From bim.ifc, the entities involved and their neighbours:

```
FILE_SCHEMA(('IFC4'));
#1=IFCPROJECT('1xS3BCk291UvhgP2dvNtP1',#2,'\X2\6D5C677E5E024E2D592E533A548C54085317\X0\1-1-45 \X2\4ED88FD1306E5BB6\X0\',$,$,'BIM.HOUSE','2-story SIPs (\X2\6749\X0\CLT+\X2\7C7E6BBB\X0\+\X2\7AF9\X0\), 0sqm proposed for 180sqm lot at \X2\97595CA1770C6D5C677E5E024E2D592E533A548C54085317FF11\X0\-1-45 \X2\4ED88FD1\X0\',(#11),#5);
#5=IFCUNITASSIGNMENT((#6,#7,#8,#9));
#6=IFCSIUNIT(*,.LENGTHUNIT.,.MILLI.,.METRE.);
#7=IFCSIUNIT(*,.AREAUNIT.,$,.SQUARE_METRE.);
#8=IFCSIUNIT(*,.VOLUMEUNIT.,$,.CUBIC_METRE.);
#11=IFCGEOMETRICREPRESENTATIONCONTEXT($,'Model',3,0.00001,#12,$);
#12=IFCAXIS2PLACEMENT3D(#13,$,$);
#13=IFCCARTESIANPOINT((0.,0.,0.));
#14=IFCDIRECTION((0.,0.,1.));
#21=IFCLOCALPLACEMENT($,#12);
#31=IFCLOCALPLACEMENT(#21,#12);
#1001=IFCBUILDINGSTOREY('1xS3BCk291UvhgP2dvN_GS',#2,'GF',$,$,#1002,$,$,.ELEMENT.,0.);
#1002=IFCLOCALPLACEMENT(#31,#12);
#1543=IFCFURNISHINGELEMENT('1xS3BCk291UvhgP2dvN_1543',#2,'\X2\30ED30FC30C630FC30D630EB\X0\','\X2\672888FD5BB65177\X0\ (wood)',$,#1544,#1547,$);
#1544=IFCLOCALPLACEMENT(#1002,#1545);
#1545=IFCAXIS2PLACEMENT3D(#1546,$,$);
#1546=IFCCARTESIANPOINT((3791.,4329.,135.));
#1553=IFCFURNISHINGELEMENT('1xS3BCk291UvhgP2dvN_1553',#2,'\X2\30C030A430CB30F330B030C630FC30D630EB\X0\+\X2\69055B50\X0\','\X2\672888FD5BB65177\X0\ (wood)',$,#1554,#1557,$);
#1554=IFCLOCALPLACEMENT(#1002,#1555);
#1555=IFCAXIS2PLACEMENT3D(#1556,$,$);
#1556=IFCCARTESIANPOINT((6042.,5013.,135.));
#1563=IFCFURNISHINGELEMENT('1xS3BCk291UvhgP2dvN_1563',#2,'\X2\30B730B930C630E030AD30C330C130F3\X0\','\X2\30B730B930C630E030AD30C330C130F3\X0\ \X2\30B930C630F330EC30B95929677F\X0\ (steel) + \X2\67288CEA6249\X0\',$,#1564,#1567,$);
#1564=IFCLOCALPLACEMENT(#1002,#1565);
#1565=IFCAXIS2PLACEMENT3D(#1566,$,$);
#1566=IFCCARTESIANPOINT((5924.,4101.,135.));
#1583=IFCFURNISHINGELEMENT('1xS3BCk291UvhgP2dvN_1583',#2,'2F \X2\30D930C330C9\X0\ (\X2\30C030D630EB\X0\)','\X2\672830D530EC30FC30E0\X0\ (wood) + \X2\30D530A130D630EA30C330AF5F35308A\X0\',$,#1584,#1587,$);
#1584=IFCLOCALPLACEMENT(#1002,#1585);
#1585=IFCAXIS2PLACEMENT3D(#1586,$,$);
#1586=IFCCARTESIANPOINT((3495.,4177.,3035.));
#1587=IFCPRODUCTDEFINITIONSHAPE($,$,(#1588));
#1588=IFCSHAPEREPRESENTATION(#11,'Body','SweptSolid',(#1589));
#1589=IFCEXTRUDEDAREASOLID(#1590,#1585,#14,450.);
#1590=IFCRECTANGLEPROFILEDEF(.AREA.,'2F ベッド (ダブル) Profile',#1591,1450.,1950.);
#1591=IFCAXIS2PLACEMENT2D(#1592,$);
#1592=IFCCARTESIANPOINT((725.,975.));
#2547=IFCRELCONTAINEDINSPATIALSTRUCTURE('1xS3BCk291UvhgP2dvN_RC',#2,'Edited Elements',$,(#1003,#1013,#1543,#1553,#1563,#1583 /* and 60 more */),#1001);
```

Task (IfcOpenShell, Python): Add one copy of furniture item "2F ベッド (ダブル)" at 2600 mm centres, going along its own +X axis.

```python
import ifcopenshell
import ifcopenshell.api.geometry
import ifcopenshell.api.root
import ifcopenshell.util.element
import ifcopenshell.util.placement
import ifcopenshell.util.unit

model = ifcopenshell.open("bim.ifc")
unit_scale = ifcopenshell.util.unit.calculate_unit_scale(model)


def reuse_history(source, copy):
    """copy_class also copies each property set's owner history, people and application; keep the originals."""
    for rel in copy.IsDefinedBy:
        if rel.is_a("IfcRelDefinesByProperties") and (history := rel.RelatingPropertyDefinition.OwnerHistory):
            rel.RelatingPropertyDefinition.OwnerHistory = source.OwnerHistory
            ifcopenshell.util.element.remove_deep2(model, history)


source = model.by_id(1583)
base = ifcopenshell.util.placement.get_local_placement(source.ObjectPlacement)
step = base[:3, 0] * 2.6 / unit_scale

for i in range(1, 2):
    copy = ifcopenshell.api.root.copy_class(model, product=source)
    copy.Representation = ifcopenshell.util.element.copy_deep(
        model, source.Representation, exclude=["IfcGeometricRepresentationContext", "IfcRepresentationMap"]
    )
    reuse_history(source, copy)
    matrix = base.copy()
    matrix[:3, 3] += i * step
    print("added at", matrix[:3, 3].round(3) + 0.0)
    ifcopenshell.api.geometry.edit_object_placement(model, product=copy, matrix=matrix, is_si=False)

model.write("bim_rev.ifc")
```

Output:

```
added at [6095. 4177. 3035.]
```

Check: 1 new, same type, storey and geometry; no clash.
